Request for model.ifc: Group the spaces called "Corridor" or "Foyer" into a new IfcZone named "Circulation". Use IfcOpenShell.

First a look at what the model holds.

```python
import ifcopenshell

model = ifcopenshell.open("model.ifc")
print(model.schema)
seen = {}
for space in model.by_type("IfcSpace"):
    seen[space.LongName] = seen.get(space.LongName, 0) + 1
for name, count in sorted(seen.items(), key=str):
    print(count, "x", name)
print("zones:", [z.Name for z in model.by_type("IfcZone")][:20])
```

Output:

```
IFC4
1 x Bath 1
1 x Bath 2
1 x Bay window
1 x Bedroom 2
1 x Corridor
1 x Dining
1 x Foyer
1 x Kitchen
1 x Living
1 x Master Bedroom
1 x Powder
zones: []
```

```python
import ifcopenshell
import ifcopenshell.api.group
import ifcopenshell.api.root

model = ifcopenshell.open("model.ifc")

names = {"Corridor", "Foyer"}
spaces = [s for s in model.by_type("IfcSpace") if s.LongName in names]

zone = ifcopenshell.api.root.create_entity(model, ifc_class="IfcZone", name="Circulation")
ifcopenshell.api.group.assign_group(model, products=spaces, group=zone)
print(len(spaces), "spaces in", zone.Name)

model.write("model-out.ifc")
```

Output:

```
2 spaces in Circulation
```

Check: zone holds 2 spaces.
